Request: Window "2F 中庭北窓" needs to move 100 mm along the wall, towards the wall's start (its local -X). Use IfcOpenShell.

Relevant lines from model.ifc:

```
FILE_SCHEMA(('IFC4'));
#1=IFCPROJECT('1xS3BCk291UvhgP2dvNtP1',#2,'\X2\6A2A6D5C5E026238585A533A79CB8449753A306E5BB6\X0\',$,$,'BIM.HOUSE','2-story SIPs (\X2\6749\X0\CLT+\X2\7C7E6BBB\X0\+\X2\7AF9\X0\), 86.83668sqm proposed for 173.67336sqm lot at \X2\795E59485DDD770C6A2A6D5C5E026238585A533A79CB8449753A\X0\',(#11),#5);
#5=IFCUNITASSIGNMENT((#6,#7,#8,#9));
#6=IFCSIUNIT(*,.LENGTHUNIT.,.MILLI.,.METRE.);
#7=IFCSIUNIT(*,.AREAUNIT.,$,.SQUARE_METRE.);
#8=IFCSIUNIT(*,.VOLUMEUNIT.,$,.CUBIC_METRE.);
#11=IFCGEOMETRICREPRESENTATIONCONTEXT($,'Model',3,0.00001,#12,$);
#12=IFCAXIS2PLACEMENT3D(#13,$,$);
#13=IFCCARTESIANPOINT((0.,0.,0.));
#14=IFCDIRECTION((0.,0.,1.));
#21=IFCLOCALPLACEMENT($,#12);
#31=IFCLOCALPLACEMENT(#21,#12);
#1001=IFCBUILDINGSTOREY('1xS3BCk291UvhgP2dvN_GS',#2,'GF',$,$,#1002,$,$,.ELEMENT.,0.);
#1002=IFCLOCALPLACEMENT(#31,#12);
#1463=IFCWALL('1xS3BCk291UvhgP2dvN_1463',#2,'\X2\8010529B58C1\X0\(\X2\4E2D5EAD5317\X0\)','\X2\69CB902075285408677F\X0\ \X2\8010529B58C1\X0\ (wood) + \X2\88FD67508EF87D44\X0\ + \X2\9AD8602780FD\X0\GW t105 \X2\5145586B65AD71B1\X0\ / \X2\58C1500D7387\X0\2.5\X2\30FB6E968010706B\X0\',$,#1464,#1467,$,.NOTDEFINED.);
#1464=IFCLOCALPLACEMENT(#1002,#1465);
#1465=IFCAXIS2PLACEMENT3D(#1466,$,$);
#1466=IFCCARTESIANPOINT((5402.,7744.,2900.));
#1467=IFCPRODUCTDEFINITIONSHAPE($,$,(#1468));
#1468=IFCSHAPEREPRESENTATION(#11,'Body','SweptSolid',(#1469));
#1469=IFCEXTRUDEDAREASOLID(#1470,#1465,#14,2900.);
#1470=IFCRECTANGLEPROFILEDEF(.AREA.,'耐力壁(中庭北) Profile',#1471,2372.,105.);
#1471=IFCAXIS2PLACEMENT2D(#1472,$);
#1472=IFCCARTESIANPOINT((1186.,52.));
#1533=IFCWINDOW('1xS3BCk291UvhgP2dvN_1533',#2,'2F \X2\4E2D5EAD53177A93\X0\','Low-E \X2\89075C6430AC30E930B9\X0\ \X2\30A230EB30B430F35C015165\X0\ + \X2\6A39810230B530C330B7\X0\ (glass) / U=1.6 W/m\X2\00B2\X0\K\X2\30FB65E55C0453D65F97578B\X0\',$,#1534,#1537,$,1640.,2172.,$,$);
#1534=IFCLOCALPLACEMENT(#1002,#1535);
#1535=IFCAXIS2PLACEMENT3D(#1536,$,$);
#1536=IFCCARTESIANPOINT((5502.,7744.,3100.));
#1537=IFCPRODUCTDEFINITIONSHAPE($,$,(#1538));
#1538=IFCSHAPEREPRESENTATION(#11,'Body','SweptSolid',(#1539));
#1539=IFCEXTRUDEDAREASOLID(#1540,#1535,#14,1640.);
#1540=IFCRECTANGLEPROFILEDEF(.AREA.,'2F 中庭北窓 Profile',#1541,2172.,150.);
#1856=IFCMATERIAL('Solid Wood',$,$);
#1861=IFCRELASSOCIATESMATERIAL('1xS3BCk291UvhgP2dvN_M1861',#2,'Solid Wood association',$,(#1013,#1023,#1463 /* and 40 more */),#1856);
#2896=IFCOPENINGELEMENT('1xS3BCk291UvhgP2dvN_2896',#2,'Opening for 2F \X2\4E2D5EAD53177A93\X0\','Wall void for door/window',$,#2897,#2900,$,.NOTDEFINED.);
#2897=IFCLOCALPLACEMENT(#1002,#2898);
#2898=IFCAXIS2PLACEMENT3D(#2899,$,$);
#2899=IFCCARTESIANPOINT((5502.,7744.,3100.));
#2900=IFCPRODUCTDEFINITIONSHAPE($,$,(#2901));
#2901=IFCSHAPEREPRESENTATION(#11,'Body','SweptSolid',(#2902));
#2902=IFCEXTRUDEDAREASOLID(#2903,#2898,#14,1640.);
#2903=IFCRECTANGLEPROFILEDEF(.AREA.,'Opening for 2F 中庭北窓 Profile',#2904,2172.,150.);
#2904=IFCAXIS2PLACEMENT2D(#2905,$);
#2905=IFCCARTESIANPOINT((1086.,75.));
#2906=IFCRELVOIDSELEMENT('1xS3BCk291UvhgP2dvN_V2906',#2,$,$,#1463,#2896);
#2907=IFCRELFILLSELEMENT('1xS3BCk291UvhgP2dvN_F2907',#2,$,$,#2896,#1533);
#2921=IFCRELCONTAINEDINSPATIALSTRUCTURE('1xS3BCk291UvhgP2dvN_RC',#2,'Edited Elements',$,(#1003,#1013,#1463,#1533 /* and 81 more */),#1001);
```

```python
import ifcopenshell
import ifcopenshell.api.geometry
import ifcopenshell.util.placement

model = ifcopenshell.open("model.ifc")

window = model.by_guid("1xS3BCk291UvhgP2dvN_1533")
opening = window.FillsVoids[0].RelatingOpeningElement
wall = opening.VoidsElements[0].RelatingBuildingElement

wall_matrix = ifcopenshell.util.placement.get_local_placement(wall.ObjectPlacement)
shift = wall_matrix[:3, 0] * -100.0
before = ifcopenshell.util.placement.get_local_placement(window.ObjectPlacement)[:3, 3].copy()

# The window is not placed relative to its opening, so move both.
for product in (opening, window):
    matrix = ifcopenshell.util.placement.get_local_placement(product.ObjectPlacement)
    matrix[:3, 3] += shift
    ifcopenshell.api.geometry.edit_object_placement(model, product=product, matrix=matrix, is_si=False)

after = ifcopenshell.util.placement.get_local_placement(window.ObjectPlacement)[:3, 3]
print("window moved by", (after - before).round(3) + 0.0)

model.write("model_v2.ifc")
```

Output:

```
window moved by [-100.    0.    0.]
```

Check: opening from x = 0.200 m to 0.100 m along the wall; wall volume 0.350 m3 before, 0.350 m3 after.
